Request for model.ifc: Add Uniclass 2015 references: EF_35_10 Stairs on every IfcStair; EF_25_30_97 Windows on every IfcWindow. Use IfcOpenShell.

First a look at what the model holds.

```python
import ifcopenshell

model = ifcopenshell.open("model.ifc")
print(model.schema)
print("classifications:", [c.Name for c in model.by_type("IfcClassification")])
for ifc_class in ("IfcDoor", "IfcRoof", "IfcStair", "IfcWall", "IfcWindow"):
    print(ifc_class, len(model.by_type(ifc_class)))
```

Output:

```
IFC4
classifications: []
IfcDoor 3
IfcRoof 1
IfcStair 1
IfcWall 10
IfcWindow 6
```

```python
import ifcopenshell
import ifcopenshell.api.classification

model = ifcopenshell.open("model.ifc")

system = ifcopenshell.api.classification.add_classification(model, classification="Uniclass 2015")

codes = {
    "IfcStair": ("EF_35_10", "Stairs"),
    "IfcWindow": ("EF_25_30_97", "Windows"),
}
for ifc_class, (code, name) in codes.items():
    products = model.by_type(ifc_class)
    ifcopenshell.api.classification.add_reference(
        model, products=products, classification=system, identification=code, name=name
    )
    print(code, len(products))

model.write("model-out.ifc")
```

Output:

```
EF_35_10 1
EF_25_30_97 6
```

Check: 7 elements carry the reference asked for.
